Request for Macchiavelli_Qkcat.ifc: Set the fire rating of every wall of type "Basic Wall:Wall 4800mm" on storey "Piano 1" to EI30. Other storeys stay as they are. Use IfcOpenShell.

First a look at what the model holds.

```python
import ifcopenshell
import ifcopenshell.util.element

model = ifcopenshell.open("Macchiavelli_Qkcat.ifc")
print(model.schema)
storey = next(s for s in model.by_type("IfcBuildingStorey") if s.Name == "Piano 1")
walls = [e for e in ifcopenshell.util.element.get_decomposition(storey) if e.is_a("IfcWall")]
seen = {}
for e in walls:
    element_type = ifcopenshell.util.element.get_type(e)
    key = (element_type.Name if element_type != e and element_type else None, ifcopenshell.util.element.get_pset(e, "Pset_WallCommon", "FireRating"))
    seen[key] = seen.get(key, 0) + 1
for (name, value), count in sorted(seen.items(), key=str):
    print(count, "x", name, "|", value)
```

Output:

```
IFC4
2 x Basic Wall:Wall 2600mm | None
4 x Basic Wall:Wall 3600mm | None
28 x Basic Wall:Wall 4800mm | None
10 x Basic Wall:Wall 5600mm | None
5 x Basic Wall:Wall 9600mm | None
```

```python
import ifcopenshell
import ifcopenshell.api.pset
import ifcopenshell.util.element

model = ifcopenshell.open("Macchiavelli_Qkcat.ifc")

storey = next(s for s in model.by_type("IfcBuildingStorey") if s.Name == "Piano 1")
walls = [e for e in ifcopenshell.util.element.get_decomposition(storey) if e.is_a("IfcWall")]

count = 0
for e in walls:
    element_type = ifcopenshell.util.element.get_type(e)
    if element_type in (None, e) or element_type.Name != "Basic Wall:Wall 4800mm":
        continue
    # add_pset returns the element's existing set when there is one.
    pset = ifcopenshell.api.pset.add_pset(model, product=e, name="Pset_WallCommon")
    ifcopenshell.api.pset.edit_pset(model, pset=pset, properties={"FireRating": "EI30"})
    count += 1

print(count, "walls updated")

model.write("Macchiavelli_Qkcat_rev.ifc")
```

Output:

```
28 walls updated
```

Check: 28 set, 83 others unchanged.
